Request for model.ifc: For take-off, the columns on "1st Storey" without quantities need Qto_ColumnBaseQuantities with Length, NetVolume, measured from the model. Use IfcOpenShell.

First a look at what the model holds.

```python
import ifcopenshell
import ifcopenshell.util.element
import ifcopenshell.util.unit

model = ifcopenshell.open("model.ifc")
print(model.schema)
for unit_type in ("LENGTHUNIT", "AREAUNIT", "VOLUMEUNIT"):
    print(unit_type, ifcopenshell.util.unit.calculate_unit_scale(model, unit_type))
storey = next(s for s in model.by_type("IfcBuildingStorey") if s.Name == "1st Storey")
columns = [e for e in ifcopenshell.util.element.get_decomposition(storey) if e.is_a("IfcColumn")]
for e in sorted(columns, key=lambda e: e.id()):
    print(e.id(), e.is_a(), e.Name, list(ifcopenshell.util.element.get_psets(e, qtos_only=True)), sep=" | ")
```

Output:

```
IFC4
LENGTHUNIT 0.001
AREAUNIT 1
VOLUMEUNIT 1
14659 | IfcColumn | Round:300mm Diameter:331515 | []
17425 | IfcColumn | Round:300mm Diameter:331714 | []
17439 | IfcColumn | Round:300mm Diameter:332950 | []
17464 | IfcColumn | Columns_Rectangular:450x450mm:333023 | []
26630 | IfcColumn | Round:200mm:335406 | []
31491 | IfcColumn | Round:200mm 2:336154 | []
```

```python
import ifcopenshell
import ifcopenshell.api.pset
import ifcopenshell.geom
import ifcopenshell.util.element
import ifcopenshell.util.shape
import ifcopenshell.util.unit

model = ifcopenshell.open("model.ifc")
unit_scale = ifcopenshell.util.unit.calculate_unit_scale(model)
volume_scale = ifcopenshell.util.unit.calculate_unit_scale(model, "VOLUMEUNIT")
settings = ifcopenshell.geom.settings()

storey = next(s for s in model.by_type("IfcBuildingStorey") if s.Name == "1st Storey")
columns = [e for e in ifcopenshell.util.element.get_decomposition(storey) if e.is_a("IfcColumn")]

for e in sorted(columns, key=lambda e: e.id()):
    if ifcopenshell.util.element.get_psets(e, qtos_only=True, should_inherit=False):
        continue
    # Geometry comes back in metres, in the element's own axes.
    shape = ifcopenshell.geom.create_shape(settings, e)
    values = {
        "Length": ifcopenshell.util.shape.get_z(shape.geometry) / unit_scale,
        "NetVolume": ifcopenshell.util.shape.get_volume(shape.geometry) / volume_scale,
    }
    qto = ifcopenshell.api.pset.add_qto(model, product=e, name="Qto_ColumnBaseQuantities")
    ifcopenshell.api.pset.edit_qto(model, qto=qto, properties=values)
    print(e.id(), {k: round(v, 3) for k, v in values.items()})

model.write("model_v2.ifc")
```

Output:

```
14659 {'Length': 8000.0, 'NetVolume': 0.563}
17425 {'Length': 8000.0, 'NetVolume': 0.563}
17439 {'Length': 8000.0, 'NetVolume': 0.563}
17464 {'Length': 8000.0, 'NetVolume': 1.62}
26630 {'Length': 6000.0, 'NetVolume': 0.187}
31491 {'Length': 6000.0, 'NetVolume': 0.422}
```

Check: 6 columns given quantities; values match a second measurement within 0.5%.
